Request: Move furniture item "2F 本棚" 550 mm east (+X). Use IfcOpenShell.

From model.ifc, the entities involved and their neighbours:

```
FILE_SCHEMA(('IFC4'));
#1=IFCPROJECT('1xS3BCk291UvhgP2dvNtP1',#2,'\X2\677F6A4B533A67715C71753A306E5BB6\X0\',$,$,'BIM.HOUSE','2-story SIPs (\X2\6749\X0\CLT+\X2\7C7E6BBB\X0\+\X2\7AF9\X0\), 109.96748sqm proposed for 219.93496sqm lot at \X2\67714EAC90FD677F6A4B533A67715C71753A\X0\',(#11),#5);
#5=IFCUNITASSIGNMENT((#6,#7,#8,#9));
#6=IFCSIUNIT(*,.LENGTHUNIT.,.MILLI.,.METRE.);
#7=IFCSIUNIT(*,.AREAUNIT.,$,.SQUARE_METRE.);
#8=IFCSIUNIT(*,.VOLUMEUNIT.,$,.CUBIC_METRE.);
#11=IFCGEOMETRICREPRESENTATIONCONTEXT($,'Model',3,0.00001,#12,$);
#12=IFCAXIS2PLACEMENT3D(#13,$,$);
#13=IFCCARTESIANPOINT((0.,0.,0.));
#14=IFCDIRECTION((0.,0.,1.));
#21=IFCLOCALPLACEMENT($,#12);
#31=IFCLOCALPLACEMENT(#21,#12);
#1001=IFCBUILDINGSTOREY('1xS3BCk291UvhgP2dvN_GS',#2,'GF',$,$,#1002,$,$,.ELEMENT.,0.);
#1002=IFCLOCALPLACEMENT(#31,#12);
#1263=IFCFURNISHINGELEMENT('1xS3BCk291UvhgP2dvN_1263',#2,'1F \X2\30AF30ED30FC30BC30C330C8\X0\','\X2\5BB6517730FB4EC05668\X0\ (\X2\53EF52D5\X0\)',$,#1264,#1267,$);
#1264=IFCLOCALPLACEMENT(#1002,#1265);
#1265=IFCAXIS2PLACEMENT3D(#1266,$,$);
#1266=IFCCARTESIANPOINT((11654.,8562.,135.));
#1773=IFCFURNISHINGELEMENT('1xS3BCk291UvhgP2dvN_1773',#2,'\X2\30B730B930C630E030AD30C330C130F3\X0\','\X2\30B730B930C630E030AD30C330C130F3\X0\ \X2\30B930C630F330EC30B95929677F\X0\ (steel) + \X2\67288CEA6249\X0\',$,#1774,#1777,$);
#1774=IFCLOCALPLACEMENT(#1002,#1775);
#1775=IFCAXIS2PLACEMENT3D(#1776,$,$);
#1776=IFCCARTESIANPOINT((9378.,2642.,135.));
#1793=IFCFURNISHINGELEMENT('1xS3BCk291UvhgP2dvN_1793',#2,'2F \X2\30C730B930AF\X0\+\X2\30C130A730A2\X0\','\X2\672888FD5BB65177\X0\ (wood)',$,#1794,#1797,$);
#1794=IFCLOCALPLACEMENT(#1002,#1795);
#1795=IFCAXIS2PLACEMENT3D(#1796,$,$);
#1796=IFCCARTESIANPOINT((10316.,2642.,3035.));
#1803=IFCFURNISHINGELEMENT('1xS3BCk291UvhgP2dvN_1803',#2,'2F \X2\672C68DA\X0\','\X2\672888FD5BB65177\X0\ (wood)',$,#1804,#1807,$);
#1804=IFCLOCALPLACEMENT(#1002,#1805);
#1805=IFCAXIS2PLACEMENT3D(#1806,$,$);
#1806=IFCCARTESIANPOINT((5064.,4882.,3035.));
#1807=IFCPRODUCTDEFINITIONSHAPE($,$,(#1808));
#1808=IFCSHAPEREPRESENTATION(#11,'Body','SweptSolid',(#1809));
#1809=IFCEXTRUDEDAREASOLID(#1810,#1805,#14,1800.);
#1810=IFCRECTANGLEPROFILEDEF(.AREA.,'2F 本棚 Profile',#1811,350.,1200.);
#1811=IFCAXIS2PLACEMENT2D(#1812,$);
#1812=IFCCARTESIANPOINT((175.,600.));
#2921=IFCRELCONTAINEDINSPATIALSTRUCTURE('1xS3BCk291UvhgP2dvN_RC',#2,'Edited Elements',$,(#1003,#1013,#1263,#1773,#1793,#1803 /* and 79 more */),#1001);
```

```python
import ifcopenshell
import ifcopenshell.api.geometry
import ifcopenshell.util.placement
import ifcopenshell.util.unit

model = ifcopenshell.open("model.ifc")
unit_scale = ifcopenshell.util.unit.calculate_unit_scale(model)

item = model.by_guid("1xS3BCk291UvhgP2dvN_1803")
matrix = ifcopenshell.util.placement.get_local_placement(item.ObjectPlacement)
matrix[0, 3] += 0.55 / unit_scale
ifcopenshell.api.geometry.edit_object_placement(model, product=item, matrix=matrix, is_si=False)

print(ifcopenshell.util.placement.get_local_placement(item.ObjectPlacement).round(3) + 0.0)

model.write("model-out.ifc")
```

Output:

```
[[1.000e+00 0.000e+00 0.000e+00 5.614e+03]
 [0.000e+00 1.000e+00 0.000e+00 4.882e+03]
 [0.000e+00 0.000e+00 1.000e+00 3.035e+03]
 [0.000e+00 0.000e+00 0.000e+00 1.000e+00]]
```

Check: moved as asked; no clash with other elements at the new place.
